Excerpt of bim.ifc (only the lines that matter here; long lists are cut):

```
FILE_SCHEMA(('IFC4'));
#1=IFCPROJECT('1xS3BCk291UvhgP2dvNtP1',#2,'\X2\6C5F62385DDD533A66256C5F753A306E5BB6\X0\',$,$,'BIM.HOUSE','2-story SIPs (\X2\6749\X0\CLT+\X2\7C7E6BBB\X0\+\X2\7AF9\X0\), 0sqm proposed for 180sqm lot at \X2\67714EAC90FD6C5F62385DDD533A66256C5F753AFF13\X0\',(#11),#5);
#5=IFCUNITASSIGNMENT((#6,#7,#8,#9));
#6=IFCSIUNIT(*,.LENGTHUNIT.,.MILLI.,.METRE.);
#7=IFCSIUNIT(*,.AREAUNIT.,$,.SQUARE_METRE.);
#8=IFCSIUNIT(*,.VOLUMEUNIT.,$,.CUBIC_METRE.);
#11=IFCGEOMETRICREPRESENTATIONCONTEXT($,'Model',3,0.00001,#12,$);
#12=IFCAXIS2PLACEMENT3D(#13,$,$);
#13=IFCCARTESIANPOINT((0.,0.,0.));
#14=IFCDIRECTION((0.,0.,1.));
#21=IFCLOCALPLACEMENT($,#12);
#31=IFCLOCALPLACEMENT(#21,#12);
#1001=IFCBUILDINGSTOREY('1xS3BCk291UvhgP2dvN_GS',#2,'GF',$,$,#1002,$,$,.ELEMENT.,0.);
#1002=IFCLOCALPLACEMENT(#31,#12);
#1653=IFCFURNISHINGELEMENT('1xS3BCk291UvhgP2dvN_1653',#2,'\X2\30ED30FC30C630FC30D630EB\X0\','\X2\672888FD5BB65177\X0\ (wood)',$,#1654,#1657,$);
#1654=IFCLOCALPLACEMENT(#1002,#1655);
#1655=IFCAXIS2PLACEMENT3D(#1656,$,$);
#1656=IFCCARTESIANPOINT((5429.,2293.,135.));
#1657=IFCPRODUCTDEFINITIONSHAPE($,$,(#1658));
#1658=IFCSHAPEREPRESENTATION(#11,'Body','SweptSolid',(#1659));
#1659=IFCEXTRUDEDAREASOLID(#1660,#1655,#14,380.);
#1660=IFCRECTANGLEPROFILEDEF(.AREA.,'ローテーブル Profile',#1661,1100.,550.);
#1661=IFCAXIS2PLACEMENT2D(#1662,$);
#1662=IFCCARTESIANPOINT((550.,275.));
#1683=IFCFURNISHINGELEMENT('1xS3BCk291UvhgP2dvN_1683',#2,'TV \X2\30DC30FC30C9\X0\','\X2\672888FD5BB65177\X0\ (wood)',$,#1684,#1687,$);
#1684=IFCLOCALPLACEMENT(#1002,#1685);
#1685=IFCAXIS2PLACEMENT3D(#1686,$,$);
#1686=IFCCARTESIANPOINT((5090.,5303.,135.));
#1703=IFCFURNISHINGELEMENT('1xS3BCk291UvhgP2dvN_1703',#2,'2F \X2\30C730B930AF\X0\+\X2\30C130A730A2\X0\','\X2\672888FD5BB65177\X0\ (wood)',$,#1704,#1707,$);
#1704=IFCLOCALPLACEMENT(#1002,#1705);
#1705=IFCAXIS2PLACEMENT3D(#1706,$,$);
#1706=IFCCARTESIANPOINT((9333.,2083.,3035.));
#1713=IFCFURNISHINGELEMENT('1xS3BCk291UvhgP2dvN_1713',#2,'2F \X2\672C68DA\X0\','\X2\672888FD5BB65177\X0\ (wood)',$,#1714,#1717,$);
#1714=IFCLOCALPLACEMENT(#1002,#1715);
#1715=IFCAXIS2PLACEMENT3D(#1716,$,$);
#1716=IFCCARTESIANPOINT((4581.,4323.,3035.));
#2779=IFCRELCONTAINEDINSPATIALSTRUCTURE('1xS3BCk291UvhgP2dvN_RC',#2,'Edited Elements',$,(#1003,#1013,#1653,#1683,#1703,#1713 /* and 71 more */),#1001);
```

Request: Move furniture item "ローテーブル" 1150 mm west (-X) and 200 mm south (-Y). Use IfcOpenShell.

```python
import ifcopenshell
import ifcopenshell.api.geometry
import ifcopenshell.util.placement

model = ifcopenshell.open("bim.ifc")

item = model.by_guid("1xS3BCk291UvhgP2dvN_1653")
matrix = ifcopenshell.util.placement.get_local_placement(item.ObjectPlacement)
matrix[0, 3] -= 1150.0
matrix[1, 3] -= 200.0
ifcopenshell.api.geometry.edit_object_placement(model, product=item, matrix=matrix, is_si=False)

print(ifcopenshell.util.placement.get_local_placement(item.ObjectPlacement).round(3) + 0.0)

model.write("bim_updated.ifc")
```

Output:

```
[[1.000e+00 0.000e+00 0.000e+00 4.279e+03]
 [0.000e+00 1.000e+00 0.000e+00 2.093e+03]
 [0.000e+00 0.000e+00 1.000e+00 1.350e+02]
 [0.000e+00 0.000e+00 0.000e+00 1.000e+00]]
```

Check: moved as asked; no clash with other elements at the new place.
